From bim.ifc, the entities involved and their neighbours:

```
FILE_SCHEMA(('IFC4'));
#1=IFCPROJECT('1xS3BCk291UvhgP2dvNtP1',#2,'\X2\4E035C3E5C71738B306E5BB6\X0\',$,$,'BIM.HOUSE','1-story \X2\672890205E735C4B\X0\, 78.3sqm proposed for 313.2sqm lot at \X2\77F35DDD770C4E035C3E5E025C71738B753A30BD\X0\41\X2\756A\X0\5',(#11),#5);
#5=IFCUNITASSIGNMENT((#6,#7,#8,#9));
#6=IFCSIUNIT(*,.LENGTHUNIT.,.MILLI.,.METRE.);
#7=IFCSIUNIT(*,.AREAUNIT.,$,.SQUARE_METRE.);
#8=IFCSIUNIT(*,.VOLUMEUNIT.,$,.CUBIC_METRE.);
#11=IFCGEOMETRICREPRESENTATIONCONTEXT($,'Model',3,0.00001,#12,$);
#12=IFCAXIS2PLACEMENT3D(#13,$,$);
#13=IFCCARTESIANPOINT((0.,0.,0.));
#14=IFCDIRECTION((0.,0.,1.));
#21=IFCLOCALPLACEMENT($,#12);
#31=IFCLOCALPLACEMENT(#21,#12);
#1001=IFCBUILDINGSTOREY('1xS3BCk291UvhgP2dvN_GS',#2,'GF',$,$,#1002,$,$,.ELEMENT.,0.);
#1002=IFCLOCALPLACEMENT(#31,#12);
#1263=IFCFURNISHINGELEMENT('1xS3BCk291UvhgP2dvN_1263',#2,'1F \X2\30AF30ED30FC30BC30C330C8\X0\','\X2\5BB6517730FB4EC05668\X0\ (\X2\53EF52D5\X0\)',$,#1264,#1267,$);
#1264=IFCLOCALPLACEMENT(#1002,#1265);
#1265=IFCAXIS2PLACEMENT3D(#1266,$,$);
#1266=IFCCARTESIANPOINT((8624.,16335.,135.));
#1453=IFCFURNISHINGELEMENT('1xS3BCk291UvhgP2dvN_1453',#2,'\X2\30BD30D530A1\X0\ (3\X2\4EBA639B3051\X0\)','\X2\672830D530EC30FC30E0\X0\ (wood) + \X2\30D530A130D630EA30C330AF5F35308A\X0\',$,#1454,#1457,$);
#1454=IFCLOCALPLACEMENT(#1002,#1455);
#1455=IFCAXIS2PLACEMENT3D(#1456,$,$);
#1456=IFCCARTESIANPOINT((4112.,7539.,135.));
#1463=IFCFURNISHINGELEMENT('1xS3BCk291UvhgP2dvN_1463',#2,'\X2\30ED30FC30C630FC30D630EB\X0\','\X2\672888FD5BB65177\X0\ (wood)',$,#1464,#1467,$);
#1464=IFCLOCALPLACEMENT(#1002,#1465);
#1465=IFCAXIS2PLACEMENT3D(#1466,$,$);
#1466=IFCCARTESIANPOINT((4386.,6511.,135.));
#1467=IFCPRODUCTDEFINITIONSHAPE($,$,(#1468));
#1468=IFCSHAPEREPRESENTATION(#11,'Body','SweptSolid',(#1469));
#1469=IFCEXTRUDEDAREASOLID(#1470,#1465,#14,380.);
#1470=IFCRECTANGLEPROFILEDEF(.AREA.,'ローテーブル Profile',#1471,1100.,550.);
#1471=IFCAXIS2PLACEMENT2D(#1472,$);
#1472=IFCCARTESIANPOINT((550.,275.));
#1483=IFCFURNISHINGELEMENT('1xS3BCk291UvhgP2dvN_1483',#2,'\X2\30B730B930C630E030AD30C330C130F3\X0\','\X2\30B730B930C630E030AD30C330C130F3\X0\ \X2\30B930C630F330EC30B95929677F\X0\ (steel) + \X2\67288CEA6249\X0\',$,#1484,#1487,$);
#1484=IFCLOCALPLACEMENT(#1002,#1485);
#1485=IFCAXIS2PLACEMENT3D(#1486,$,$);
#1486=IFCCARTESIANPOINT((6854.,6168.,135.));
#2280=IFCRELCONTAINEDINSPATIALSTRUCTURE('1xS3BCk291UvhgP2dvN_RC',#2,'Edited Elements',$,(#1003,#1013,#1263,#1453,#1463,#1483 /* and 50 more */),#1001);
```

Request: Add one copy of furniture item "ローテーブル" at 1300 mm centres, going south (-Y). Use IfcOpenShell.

```python
import numpy as np
import ifcopenshell
import ifcopenshell.api.geometry
import ifcopenshell.api.root
import ifcopenshell.util.element
import ifcopenshell.util.placement
import ifcopenshell.util.unit

model = ifcopenshell.open("bim.ifc")
unit_scale = ifcopenshell.util.unit.calculate_unit_scale(model)


def reuse_history(source, copy):
    """copy_class also copies each property set's owner history, people and application; keep the originals."""
    for rel in copy.IsDefinedBy:
        if rel.is_a("IfcRelDefinesByProperties") and (history := rel.RelatingPropertyDefinition.OwnerHistory):
            rel.RelatingPropertyDefinition.OwnerHistory = source.OwnerHistory
            ifcopenshell.util.element.remove_deep2(model, history)


source = model.by_guid("1xS3BCk291UvhgP2dvN_1463")
base = ifcopenshell.util.placement.get_local_placement(source.ObjectPlacement)
step = np.array([0.0, -1.0, 0.0]) * 1.3 / unit_scale

for i in range(1, 2):
    copy = ifcopenshell.api.root.copy_class(model, product=source)
    copy.Representation = ifcopenshell.util.element.copy_deep(
        model, source.Representation, exclude=["IfcGeometricRepresentationContext", "IfcRepresentationMap"]
    )
    reuse_history(source, copy)
    matrix = base.copy()
    matrix[:3, 3] += i * step
    print("added at", matrix[:3, 3].round(3) + 0.0)
    ifcopenshell.api.geometry.edit_object_placement(model, product=copy, matrix=matrix, is_si=False)

model.write("bim_edited.ifc")
```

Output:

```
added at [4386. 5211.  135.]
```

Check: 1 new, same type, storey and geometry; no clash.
